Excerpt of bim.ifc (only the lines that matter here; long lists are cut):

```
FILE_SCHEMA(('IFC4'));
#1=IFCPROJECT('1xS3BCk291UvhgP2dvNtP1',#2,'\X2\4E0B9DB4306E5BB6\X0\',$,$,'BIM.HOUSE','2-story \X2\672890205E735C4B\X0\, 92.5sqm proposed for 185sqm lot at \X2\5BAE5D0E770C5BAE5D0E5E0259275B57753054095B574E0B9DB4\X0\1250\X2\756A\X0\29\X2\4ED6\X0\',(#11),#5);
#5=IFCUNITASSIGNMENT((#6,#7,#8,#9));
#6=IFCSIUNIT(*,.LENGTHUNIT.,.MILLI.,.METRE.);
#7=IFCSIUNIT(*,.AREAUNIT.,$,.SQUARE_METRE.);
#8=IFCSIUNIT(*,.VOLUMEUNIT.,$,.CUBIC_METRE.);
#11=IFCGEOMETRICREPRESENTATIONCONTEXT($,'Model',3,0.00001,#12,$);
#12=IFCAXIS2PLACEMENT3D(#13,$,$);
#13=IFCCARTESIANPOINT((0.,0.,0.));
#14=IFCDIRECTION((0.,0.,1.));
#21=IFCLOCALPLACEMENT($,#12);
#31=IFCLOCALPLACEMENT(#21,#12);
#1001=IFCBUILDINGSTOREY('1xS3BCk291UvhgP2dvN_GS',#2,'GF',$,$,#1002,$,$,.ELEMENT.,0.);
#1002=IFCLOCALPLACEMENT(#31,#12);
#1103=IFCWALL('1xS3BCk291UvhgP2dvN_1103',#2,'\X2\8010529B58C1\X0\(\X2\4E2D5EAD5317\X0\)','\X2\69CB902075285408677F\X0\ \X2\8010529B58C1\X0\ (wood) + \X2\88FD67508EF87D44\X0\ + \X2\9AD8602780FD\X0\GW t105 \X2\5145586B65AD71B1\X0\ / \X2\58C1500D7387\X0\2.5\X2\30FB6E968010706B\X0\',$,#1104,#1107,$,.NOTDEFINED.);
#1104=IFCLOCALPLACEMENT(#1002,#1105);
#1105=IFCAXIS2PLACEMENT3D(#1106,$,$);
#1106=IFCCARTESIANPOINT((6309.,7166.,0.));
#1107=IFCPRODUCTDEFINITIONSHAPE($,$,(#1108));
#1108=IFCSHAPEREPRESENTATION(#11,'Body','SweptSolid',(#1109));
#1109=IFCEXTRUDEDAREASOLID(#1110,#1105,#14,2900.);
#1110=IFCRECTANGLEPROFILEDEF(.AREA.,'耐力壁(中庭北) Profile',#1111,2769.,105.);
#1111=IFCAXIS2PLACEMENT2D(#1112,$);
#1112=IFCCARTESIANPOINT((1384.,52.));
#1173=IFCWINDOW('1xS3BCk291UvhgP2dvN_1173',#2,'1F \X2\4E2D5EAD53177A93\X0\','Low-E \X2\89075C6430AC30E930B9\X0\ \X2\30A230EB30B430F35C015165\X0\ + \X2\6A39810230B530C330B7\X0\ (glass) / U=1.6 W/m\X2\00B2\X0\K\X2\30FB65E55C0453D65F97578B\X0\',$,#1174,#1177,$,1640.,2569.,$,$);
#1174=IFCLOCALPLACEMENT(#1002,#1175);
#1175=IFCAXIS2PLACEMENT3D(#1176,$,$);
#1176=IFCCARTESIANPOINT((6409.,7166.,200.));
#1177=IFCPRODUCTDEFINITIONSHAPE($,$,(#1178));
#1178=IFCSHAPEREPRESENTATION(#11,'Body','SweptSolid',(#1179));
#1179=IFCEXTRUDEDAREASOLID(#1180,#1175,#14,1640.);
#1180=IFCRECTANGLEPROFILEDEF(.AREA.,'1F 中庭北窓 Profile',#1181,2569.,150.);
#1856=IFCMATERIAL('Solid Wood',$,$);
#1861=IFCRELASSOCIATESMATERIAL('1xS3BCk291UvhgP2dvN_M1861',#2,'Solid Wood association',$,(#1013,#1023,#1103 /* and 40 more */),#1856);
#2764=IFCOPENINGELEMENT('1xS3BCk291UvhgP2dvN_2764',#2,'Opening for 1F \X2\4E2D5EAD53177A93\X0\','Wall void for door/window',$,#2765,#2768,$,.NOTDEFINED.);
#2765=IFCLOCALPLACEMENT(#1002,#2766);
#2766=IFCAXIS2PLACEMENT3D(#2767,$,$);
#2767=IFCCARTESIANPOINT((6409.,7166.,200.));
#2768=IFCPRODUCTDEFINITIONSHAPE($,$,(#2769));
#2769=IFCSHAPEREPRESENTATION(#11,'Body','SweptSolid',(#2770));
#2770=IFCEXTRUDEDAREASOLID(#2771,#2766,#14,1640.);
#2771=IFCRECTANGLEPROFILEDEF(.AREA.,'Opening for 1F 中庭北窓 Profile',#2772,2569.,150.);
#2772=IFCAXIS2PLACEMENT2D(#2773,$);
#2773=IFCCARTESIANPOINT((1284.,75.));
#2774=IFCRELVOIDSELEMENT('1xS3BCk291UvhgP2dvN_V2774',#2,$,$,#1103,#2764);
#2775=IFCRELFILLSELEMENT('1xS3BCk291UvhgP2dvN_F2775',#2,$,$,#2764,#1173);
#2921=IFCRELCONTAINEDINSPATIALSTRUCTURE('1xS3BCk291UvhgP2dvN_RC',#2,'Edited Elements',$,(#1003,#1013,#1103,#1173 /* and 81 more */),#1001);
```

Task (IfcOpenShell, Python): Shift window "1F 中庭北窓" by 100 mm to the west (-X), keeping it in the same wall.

```python
import ifcopenshell
import ifcopenshell.api.geometry
import ifcopenshell.util.placement
import ifcopenshell.util.unit

model = ifcopenshell.open("bim.ifc")
unit_scale = ifcopenshell.util.unit.calculate_unit_scale(model)

window = model.by_guid("1xS3BCk291UvhgP2dvN_1173")
opening = window.FillsVoids[0].RelatingOpeningElement
wall = opening.VoidsElements[0].RelatingBuildingElement

wall_matrix = ifcopenshell.util.placement.get_local_placement(wall.ObjectPlacement)
shift = wall_matrix[:3, 0] * -0.1 / unit_scale
before = ifcopenshell.util.placement.get_local_placement(window.ObjectPlacement)[:3, 3].copy()

# The window is not placed relative to its opening, so move both.
for product in (opening, window):
    matrix = ifcopenshell.util.placement.get_local_placement(product.ObjectPlacement)
    matrix[:3, 3] += shift
    ifcopenshell.api.geometry.edit_object_placement(model, product=product, matrix=matrix, is_si=False)

after = ifcopenshell.util.placement.get_local_placement(window.ObjectPlacement)[:3, 3]
print("window moved by", (after - before).round(3) + 0.0)

model.write("bim-out.ifc")
```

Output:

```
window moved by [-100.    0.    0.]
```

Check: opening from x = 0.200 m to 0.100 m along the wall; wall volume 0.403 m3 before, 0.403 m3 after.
